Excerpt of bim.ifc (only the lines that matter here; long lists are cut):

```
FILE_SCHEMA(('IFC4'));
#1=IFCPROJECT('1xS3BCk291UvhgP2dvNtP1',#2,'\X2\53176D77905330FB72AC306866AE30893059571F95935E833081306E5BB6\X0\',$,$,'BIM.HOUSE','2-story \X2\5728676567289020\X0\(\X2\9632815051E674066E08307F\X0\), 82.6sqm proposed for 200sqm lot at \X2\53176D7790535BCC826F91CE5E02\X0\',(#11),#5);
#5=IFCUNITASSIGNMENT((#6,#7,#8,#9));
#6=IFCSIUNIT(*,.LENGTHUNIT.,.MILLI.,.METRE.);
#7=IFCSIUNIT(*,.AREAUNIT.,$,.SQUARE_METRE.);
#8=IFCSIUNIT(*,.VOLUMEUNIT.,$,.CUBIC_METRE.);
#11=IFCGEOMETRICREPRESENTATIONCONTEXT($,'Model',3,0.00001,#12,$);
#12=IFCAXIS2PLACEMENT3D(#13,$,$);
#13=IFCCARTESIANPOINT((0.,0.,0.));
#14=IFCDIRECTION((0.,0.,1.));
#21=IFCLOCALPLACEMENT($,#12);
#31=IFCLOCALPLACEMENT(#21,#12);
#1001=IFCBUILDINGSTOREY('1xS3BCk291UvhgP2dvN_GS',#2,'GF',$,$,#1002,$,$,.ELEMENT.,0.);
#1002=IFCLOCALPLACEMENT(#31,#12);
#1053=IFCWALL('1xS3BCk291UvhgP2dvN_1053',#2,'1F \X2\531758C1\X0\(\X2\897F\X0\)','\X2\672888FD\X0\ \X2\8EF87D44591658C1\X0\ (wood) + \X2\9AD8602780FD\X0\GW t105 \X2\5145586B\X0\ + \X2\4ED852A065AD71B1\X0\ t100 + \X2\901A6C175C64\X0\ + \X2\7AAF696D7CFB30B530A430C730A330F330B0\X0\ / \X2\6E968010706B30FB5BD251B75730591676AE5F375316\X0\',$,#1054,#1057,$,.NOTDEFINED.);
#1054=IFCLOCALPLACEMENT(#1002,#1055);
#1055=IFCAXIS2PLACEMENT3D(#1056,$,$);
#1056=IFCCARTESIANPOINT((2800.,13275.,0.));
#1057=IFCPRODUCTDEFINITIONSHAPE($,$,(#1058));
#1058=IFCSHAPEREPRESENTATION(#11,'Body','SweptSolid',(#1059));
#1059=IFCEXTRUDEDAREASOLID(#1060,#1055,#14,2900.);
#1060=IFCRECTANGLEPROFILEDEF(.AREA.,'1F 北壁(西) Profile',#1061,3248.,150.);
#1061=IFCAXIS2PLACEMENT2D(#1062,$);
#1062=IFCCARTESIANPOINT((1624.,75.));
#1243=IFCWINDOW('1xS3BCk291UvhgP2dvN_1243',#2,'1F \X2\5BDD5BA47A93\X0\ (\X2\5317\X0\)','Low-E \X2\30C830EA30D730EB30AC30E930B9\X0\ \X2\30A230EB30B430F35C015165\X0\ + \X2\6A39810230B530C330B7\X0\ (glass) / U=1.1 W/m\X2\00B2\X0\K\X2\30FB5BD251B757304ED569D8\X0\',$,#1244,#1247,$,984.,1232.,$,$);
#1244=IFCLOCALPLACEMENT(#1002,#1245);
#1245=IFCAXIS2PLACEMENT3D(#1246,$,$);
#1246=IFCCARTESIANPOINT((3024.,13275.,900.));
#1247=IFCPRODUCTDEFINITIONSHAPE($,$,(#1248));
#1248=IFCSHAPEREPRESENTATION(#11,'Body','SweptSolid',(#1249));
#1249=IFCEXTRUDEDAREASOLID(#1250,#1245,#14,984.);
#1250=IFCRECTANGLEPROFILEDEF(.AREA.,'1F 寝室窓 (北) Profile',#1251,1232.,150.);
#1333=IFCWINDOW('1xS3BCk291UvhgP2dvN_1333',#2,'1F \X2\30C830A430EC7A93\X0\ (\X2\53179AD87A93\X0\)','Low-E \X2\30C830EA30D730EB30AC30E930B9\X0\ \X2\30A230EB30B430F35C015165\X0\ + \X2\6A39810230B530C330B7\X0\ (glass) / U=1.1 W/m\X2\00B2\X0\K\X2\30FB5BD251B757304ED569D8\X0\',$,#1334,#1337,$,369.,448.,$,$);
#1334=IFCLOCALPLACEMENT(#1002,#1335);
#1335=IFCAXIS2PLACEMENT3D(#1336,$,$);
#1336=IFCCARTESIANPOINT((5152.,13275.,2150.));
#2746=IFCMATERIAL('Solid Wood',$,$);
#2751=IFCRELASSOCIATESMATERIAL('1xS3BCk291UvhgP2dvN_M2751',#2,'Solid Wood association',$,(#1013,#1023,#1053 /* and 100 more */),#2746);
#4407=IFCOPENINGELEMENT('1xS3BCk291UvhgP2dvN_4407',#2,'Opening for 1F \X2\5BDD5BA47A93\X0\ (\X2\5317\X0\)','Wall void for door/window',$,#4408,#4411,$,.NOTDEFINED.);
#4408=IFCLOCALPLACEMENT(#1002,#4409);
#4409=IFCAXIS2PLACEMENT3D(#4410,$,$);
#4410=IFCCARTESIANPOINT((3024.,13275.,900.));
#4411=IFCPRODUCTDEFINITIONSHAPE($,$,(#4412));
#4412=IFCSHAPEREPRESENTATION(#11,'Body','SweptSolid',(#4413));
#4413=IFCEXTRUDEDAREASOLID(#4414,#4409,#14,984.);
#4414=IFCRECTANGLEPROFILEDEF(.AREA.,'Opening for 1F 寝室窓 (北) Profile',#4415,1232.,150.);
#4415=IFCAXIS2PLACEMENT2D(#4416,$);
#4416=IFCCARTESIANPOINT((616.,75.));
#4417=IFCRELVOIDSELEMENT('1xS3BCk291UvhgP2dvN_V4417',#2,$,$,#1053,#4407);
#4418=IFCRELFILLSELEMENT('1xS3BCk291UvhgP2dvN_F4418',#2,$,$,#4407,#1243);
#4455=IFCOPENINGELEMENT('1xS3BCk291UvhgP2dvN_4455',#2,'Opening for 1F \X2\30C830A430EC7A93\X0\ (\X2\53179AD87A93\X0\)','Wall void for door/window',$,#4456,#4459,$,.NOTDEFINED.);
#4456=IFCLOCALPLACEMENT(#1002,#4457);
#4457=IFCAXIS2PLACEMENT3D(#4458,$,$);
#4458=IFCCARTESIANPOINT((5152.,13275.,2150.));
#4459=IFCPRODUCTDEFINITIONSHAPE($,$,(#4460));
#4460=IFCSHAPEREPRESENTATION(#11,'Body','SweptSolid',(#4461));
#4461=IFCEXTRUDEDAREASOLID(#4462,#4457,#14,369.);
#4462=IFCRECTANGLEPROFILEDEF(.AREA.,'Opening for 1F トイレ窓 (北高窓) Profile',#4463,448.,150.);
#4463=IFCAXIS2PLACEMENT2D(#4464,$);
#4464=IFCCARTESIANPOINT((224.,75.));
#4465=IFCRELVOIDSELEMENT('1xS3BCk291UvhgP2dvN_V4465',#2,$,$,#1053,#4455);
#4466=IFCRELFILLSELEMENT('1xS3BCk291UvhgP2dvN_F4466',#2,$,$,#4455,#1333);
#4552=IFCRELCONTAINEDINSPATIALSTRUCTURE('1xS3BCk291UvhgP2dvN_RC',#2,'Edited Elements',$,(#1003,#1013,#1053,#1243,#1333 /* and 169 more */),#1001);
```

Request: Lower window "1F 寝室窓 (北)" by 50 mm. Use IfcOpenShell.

```python
import numpy as np
import ifcopenshell
import ifcopenshell.api.geometry
import ifcopenshell.util.placement
import ifcopenshell.util.unit

model = ifcopenshell.open("bim.ifc")
unit_scale = ifcopenshell.util.unit.calculate_unit_scale(model)

window = model.by_id(1243)
opening = window.FillsVoids[0].RelatingOpeningElement
dz = -0.05 / unit_scale

shift = np.array([0.0, 0.0, dz])
# The window is not placed relative to its opening, so move both.
for product in (opening, window):
    matrix = ifcopenshell.util.placement.get_local_placement(product.ObjectPlacement)
    matrix[:3, 3] += shift
    ifcopenshell.api.geometry.edit_object_placement(model, product=product, matrix=matrix, is_si=False)

print(f"moved by {dz * unit_scale:+.3f} m")

model.write("bim_updated.ifc")
```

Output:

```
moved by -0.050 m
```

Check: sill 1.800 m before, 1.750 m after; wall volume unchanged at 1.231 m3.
